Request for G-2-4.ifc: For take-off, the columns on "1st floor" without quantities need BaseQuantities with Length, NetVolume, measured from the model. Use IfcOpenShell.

First a look at what the model holds.

```python
import ifcopenshell
import ifcopenshell.util.element
import ifcopenshell.util.unit

model = ifcopenshell.open("G-2-4.ifc")
print(model.schema)
for unit_type in ("LENGTHUNIT", "AREAUNIT", "VOLUMEUNIT"):
    print(unit_type, ifcopenshell.util.unit.calculate_unit_scale(model, unit_type))
storey = next(s for s in model.by_type("IfcBuildingStorey") if s.Name == "1st floor")
columns = [e for e in ifcopenshell.util.element.get_decomposition(storey) if e.is_a("IfcColumn")]
for e in sorted(columns, key=lambda e: e.id()):
    print(e.id(), e.is_a(), e.Name, list(ifcopenshell.util.element.get_psets(e, qtos_only=True)), sep=" | ")
```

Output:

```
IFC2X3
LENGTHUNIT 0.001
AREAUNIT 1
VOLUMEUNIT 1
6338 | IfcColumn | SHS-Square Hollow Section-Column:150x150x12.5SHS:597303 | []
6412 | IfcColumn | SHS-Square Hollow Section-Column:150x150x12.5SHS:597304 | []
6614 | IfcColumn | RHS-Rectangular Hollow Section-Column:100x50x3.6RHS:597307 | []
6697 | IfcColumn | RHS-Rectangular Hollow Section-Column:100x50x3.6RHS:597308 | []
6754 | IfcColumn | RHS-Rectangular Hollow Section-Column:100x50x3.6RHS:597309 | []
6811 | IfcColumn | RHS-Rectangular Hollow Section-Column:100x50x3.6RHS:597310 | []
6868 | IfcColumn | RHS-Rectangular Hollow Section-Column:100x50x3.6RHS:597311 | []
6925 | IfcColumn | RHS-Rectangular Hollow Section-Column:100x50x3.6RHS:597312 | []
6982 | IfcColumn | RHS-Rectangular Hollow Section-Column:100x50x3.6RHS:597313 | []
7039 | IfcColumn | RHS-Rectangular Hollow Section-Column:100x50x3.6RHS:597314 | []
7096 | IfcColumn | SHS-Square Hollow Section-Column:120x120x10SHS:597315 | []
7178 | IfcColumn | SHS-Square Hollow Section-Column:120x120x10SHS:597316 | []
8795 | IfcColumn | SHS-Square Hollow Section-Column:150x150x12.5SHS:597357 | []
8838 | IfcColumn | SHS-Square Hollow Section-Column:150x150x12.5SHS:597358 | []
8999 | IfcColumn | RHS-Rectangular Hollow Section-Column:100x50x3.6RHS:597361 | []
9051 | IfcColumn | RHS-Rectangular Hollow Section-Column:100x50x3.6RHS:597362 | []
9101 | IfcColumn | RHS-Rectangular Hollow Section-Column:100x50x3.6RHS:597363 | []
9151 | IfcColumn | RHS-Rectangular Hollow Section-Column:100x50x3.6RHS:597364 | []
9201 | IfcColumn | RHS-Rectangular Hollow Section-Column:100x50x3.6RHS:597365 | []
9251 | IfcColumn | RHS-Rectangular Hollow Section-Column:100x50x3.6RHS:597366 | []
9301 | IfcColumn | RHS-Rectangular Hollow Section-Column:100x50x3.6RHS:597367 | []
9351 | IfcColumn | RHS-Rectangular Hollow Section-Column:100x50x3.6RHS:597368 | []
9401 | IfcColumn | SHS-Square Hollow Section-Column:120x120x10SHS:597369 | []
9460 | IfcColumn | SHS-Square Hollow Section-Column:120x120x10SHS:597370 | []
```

```python
import ifcopenshell
import ifcopenshell.api.pset
import ifcopenshell.geom
import ifcopenshell.util.element
import ifcopenshell.util.shape
import ifcopenshell.util.unit

model = ifcopenshell.open("G-2-4.ifc")
unit_scale = ifcopenshell.util.unit.calculate_unit_scale(model)
volume_scale = ifcopenshell.util.unit.calculate_unit_scale(model, "VOLUMEUNIT")
settings = ifcopenshell.geom.settings()

storey = next(s for s in model.by_type("IfcBuildingStorey") if s.Name == "1st floor")
columns = [e for e in ifcopenshell.util.element.get_decomposition(storey) if e.is_a("IfcColumn")]

for e in sorted(columns, key=lambda e: e.id()):
    if ifcopenshell.util.element.get_psets(e, qtos_only=True, should_inherit=False):
        continue
    # Geometry comes back in metres, in the element's own axes.
    shape = ifcopenshell.geom.create_shape(settings, e)
    values = {
        "Length": ifcopenshell.util.shape.get_z(shape.geometry) / unit_scale,
        "NetVolume": ifcopenshell.util.shape.get_volume(shape.geometry) / volume_scale,
    }
    qto = ifcopenshell.api.pset.add_qto(model, product=e, name="BaseQuantities")
    ifcopenshell.api.pset.edit_qto(model, qto=qto, properties=values)
    print(e.id(), {k: round(v, 3) for k, v in values.items()})

model.write("G-2-4_v2.ifc")
```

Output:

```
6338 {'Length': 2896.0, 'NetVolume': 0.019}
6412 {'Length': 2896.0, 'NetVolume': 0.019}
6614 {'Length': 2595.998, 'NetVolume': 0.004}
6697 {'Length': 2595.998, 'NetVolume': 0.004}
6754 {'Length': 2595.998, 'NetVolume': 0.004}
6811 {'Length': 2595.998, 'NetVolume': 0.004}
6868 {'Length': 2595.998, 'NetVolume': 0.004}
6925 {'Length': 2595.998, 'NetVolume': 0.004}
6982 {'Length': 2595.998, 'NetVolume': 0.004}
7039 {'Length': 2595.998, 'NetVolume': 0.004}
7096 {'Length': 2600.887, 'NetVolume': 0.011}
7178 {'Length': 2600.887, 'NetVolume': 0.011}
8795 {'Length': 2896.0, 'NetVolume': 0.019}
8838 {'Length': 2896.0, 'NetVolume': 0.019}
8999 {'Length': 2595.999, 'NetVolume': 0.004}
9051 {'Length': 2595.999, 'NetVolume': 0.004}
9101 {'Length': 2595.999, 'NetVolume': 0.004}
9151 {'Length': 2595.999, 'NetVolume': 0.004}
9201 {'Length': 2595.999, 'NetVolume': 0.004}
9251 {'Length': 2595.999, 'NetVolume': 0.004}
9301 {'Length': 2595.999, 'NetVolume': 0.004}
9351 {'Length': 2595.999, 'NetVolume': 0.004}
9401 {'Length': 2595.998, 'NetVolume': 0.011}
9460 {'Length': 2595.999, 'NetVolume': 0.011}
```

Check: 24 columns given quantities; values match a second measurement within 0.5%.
